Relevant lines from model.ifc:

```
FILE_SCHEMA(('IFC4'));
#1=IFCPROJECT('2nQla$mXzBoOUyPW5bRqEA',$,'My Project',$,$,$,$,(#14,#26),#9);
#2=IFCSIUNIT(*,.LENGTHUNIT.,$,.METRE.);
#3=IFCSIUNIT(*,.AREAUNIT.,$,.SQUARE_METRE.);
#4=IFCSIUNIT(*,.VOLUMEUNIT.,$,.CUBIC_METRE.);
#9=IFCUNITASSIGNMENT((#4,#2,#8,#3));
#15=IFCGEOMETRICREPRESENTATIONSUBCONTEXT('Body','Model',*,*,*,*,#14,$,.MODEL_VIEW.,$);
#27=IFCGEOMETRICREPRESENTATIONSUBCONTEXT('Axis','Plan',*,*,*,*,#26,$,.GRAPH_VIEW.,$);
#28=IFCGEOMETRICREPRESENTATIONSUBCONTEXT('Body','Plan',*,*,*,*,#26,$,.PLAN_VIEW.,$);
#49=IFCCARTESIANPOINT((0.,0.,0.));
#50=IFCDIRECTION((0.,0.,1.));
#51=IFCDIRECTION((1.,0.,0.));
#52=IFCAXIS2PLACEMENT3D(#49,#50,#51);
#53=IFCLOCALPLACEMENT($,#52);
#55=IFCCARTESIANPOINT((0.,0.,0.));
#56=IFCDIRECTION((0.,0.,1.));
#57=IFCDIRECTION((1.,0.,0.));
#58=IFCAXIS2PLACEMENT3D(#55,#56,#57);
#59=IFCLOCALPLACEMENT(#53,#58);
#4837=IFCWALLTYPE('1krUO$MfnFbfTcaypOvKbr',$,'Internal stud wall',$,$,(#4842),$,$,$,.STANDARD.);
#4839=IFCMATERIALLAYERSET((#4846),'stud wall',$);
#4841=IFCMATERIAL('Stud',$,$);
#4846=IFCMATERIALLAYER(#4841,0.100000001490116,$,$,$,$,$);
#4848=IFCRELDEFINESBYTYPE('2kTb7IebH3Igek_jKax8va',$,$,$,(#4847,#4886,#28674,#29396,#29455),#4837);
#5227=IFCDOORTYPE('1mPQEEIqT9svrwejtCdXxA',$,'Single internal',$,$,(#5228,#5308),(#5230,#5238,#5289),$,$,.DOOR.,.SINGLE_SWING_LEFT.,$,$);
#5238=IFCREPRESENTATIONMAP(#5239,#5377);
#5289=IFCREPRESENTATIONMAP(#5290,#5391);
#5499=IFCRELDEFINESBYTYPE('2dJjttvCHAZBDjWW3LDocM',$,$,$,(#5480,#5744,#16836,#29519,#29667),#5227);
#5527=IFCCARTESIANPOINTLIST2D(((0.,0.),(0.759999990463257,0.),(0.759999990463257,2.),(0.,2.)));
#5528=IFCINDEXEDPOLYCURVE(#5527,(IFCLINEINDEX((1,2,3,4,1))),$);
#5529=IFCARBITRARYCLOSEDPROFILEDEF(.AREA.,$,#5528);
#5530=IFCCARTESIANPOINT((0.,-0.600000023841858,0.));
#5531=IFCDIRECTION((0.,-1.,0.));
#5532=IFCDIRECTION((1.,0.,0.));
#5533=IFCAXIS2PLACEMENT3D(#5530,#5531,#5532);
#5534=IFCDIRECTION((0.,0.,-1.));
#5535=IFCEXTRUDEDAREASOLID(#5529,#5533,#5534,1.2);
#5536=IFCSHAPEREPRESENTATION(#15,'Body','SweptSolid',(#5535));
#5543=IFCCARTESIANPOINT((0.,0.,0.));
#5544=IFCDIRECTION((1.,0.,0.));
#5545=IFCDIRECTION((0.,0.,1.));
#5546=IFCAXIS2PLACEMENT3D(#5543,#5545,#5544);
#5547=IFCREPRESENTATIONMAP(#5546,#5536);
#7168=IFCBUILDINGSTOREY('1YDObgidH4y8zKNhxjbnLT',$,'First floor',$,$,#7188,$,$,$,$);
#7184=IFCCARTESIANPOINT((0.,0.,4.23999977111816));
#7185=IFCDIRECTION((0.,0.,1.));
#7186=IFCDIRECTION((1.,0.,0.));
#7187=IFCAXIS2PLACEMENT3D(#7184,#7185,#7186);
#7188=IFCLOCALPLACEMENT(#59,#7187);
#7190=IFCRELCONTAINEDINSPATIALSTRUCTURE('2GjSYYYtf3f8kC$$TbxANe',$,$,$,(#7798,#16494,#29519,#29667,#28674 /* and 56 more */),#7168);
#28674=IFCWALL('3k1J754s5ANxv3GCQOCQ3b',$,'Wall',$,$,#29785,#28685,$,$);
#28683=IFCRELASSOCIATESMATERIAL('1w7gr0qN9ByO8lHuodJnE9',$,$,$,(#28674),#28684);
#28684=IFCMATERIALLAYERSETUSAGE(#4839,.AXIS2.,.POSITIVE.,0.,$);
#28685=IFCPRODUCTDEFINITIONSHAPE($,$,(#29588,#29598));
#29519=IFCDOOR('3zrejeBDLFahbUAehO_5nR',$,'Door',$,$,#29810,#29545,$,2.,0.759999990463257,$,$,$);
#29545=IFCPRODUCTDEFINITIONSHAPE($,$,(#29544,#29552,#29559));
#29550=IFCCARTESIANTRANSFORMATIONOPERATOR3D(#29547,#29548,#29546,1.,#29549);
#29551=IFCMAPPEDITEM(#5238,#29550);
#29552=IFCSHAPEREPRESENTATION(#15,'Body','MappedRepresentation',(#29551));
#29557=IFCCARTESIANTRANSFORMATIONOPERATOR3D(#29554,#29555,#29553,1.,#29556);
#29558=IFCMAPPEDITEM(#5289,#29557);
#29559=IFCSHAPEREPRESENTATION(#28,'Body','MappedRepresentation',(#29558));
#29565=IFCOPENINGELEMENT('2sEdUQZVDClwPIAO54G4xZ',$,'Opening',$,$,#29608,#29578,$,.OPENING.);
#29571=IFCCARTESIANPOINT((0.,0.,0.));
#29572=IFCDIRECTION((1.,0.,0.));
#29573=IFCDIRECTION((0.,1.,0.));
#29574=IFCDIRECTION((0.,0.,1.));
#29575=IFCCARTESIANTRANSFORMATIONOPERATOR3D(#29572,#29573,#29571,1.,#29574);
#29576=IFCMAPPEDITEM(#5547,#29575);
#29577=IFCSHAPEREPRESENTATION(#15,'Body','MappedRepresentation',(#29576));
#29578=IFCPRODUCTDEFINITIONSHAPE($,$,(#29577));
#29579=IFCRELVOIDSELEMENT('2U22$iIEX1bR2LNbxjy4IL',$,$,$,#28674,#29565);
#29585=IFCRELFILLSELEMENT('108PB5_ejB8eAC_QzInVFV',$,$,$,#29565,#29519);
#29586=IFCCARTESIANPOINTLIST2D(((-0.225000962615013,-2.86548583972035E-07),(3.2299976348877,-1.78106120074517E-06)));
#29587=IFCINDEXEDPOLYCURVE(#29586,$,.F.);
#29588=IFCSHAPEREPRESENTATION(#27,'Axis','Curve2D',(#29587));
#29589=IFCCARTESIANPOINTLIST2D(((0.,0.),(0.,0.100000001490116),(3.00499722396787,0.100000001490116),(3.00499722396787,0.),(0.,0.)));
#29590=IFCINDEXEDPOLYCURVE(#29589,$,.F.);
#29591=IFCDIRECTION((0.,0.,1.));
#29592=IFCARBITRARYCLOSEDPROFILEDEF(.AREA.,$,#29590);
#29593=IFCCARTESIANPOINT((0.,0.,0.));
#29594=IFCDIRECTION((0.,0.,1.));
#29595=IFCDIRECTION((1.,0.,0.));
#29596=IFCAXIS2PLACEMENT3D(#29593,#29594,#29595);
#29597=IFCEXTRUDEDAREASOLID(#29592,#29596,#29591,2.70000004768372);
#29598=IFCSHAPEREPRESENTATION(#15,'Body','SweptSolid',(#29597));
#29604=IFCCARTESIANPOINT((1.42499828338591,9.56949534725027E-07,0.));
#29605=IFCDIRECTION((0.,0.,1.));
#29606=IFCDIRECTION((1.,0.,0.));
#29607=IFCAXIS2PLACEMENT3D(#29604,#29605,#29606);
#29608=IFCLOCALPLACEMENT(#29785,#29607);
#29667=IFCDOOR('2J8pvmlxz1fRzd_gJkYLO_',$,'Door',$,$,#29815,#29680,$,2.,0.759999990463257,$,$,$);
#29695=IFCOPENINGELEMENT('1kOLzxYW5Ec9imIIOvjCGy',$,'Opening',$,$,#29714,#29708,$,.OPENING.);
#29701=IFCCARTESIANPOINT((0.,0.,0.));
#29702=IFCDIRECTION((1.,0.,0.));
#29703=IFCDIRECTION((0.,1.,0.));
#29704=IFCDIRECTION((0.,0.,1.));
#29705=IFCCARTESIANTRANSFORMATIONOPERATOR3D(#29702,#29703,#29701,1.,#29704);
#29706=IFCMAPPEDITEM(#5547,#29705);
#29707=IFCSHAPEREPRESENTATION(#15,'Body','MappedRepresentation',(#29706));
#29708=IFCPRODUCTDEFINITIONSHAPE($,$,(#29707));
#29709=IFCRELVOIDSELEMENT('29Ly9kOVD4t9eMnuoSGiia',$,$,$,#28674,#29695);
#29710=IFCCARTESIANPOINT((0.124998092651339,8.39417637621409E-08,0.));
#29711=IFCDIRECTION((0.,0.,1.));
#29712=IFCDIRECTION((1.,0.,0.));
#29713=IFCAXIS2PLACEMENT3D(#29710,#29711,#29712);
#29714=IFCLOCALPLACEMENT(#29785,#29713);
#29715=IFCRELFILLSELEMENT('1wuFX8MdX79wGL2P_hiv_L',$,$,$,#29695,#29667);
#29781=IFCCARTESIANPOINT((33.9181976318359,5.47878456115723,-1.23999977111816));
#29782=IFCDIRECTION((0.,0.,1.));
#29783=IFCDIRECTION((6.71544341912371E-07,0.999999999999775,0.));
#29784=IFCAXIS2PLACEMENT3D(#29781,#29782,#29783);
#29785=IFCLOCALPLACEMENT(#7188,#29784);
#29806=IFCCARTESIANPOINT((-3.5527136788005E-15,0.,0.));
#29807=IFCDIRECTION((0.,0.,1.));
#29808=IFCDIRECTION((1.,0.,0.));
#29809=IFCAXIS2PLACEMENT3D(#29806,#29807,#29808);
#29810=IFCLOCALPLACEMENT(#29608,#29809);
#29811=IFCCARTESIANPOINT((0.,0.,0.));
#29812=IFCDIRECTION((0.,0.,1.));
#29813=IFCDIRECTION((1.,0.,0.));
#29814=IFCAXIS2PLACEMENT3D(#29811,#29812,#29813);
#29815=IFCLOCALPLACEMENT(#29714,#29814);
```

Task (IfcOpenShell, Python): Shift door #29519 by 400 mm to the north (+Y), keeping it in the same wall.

```python
import ifcopenshell
import ifcopenshell.api.geometry
import ifcopenshell.util.placement
import ifcopenshell.util.unit

model = ifcopenshell.open("model.ifc")
unit_scale = ifcopenshell.util.unit.calculate_unit_scale(model)

door = model.by_guid("3zrejeBDLFahbUAehO_5nR")
opening = door.FillsVoids[0].RelatingOpeningElement
wall = opening.VoidsElements[0].RelatingBuildingElement

wall_matrix = ifcopenshell.util.placement.get_local_placement(wall.ObjectPlacement)
shift = wall_matrix[:3, 0] * 0.4 / unit_scale
before = ifcopenshell.util.placement.get_local_placement(door.ObjectPlacement)[:3, 3].copy()

# The door is placed relative to its opening, so it follows when the opening moves.
matrix = ifcopenshell.util.placement.get_local_placement(opening.ObjectPlacement)
matrix[:3, 3] += shift
ifcopenshell.api.geometry.edit_object_placement(
    model, product=opening, matrix=matrix, is_si=False, should_transform_children=True
)

after = ifcopenshell.util.placement.get_local_placement(door.ObjectPlacement)[:3, 3]
print("door moved by", (after - before).round(3) + 0.0)

model.write("model-out.ifc")
```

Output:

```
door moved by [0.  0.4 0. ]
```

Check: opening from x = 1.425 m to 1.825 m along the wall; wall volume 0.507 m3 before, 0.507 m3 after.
